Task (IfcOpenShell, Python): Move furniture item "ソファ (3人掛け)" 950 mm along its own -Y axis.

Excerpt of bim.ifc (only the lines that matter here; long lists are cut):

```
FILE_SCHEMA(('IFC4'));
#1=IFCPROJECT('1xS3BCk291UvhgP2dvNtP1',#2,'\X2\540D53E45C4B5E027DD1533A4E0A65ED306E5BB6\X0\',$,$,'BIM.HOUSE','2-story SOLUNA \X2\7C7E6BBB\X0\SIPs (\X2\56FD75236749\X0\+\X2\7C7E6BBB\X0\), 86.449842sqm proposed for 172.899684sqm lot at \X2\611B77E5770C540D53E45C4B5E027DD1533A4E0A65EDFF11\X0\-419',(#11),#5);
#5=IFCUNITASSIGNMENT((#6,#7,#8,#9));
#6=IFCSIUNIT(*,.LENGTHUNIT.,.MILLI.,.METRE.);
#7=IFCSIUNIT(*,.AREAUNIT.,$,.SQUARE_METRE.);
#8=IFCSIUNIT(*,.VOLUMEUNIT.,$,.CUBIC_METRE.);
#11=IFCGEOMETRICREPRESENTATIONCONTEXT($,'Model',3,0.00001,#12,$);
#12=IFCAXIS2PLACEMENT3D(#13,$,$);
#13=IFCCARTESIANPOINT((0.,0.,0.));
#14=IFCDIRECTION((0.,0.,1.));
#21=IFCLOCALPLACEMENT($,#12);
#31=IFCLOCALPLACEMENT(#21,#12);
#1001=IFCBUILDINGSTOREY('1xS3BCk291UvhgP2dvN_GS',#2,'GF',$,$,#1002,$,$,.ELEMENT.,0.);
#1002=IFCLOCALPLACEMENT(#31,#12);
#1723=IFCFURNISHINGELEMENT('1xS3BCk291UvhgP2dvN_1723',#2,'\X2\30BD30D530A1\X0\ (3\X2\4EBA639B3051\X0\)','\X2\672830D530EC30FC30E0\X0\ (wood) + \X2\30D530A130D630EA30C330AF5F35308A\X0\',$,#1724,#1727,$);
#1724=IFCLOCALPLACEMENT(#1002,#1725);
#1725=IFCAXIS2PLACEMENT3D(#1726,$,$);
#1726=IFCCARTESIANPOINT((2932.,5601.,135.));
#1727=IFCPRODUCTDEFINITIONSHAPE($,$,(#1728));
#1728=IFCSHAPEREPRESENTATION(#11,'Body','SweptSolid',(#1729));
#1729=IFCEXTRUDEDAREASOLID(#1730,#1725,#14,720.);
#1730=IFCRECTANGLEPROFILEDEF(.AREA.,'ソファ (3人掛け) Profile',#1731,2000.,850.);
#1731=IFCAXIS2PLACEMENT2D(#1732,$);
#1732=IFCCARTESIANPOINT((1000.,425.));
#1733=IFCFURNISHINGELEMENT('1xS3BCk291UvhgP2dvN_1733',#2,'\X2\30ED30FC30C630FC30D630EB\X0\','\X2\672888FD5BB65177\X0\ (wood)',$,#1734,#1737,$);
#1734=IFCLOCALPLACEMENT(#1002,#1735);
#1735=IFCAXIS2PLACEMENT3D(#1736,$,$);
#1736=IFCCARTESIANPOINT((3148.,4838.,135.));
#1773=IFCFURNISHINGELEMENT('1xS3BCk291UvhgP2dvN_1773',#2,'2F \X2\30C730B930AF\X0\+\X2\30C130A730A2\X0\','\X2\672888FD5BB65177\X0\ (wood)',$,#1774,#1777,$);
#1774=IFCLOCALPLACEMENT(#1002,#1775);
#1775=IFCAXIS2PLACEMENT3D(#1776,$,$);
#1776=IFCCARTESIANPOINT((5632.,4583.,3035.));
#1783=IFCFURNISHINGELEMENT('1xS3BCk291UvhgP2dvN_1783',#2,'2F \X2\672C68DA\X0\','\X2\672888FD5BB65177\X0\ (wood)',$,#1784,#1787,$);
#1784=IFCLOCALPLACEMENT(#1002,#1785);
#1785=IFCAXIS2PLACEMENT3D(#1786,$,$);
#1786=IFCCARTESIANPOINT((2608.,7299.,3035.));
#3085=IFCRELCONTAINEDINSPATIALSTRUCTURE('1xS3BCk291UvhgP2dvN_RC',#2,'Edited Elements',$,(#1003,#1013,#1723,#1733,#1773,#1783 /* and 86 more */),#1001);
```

```python
import ifcopenshell
import ifcopenshell.api.geometry
import ifcopenshell.util.placement
import ifcopenshell.util.unit

model = ifcopenshell.open("bim.ifc")
unit_scale = ifcopenshell.util.unit.calculate_unit_scale(model)

item = model.by_id(1723)
matrix = ifcopenshell.util.placement.get_local_placement(item.ObjectPlacement)
matrix[:3, 3] -= matrix[:3, 1] * 0.95 / unit_scale
ifcopenshell.api.geometry.edit_object_placement(model, product=item, matrix=matrix, is_si=False)

print(ifcopenshell.util.placement.get_local_placement(item.ObjectPlacement).round(3) + 0.0)

model.write("bim_v2.ifc")
```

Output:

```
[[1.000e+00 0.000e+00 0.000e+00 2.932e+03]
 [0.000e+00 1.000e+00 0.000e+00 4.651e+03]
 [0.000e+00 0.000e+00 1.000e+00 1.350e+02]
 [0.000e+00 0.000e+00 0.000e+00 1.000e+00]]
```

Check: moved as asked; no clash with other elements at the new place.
